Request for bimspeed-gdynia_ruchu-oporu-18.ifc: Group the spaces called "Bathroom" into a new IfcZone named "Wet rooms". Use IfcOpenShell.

First a look at what the model holds.

```python
import ifcopenshell

model = ifcopenshell.open("bimspeed-gdynia_ruchu-oporu-18.ifc")
print(model.schema)
seen = {}
for space in model.by_type("IfcSpace"):
    seen[space.LongName] = seen.get(space.LongName, 0) + 1
for name, count in sorted(seen.items(), key=str):
    print(count, "x", name)
print("zones:", [z.Name for z in model.by_type("IfcZone")][:20])
```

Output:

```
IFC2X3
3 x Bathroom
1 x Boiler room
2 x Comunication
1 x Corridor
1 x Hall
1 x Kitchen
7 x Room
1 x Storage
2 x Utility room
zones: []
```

```python
import ifcopenshell
import ifcopenshell.api.group
import ifcopenshell.api.root

model = ifcopenshell.open("bimspeed-gdynia_ruchu-oporu-18.ifc")

names = {"Bathroom"}
spaces = [s for s in model.by_type("IfcSpace") if s.LongName in names]

zone = ifcopenshell.api.root.create_entity(model, ifc_class="IfcZone", name="Wet rooms")
ifcopenshell.api.group.assign_group(model, products=spaces, group=zone)
print(len(spaces), "spaces in", zone.Name)

model.write("bimspeed-gdynia_ruchu-oporu-18_rev.ifc")
```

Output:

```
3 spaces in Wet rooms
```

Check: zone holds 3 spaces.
